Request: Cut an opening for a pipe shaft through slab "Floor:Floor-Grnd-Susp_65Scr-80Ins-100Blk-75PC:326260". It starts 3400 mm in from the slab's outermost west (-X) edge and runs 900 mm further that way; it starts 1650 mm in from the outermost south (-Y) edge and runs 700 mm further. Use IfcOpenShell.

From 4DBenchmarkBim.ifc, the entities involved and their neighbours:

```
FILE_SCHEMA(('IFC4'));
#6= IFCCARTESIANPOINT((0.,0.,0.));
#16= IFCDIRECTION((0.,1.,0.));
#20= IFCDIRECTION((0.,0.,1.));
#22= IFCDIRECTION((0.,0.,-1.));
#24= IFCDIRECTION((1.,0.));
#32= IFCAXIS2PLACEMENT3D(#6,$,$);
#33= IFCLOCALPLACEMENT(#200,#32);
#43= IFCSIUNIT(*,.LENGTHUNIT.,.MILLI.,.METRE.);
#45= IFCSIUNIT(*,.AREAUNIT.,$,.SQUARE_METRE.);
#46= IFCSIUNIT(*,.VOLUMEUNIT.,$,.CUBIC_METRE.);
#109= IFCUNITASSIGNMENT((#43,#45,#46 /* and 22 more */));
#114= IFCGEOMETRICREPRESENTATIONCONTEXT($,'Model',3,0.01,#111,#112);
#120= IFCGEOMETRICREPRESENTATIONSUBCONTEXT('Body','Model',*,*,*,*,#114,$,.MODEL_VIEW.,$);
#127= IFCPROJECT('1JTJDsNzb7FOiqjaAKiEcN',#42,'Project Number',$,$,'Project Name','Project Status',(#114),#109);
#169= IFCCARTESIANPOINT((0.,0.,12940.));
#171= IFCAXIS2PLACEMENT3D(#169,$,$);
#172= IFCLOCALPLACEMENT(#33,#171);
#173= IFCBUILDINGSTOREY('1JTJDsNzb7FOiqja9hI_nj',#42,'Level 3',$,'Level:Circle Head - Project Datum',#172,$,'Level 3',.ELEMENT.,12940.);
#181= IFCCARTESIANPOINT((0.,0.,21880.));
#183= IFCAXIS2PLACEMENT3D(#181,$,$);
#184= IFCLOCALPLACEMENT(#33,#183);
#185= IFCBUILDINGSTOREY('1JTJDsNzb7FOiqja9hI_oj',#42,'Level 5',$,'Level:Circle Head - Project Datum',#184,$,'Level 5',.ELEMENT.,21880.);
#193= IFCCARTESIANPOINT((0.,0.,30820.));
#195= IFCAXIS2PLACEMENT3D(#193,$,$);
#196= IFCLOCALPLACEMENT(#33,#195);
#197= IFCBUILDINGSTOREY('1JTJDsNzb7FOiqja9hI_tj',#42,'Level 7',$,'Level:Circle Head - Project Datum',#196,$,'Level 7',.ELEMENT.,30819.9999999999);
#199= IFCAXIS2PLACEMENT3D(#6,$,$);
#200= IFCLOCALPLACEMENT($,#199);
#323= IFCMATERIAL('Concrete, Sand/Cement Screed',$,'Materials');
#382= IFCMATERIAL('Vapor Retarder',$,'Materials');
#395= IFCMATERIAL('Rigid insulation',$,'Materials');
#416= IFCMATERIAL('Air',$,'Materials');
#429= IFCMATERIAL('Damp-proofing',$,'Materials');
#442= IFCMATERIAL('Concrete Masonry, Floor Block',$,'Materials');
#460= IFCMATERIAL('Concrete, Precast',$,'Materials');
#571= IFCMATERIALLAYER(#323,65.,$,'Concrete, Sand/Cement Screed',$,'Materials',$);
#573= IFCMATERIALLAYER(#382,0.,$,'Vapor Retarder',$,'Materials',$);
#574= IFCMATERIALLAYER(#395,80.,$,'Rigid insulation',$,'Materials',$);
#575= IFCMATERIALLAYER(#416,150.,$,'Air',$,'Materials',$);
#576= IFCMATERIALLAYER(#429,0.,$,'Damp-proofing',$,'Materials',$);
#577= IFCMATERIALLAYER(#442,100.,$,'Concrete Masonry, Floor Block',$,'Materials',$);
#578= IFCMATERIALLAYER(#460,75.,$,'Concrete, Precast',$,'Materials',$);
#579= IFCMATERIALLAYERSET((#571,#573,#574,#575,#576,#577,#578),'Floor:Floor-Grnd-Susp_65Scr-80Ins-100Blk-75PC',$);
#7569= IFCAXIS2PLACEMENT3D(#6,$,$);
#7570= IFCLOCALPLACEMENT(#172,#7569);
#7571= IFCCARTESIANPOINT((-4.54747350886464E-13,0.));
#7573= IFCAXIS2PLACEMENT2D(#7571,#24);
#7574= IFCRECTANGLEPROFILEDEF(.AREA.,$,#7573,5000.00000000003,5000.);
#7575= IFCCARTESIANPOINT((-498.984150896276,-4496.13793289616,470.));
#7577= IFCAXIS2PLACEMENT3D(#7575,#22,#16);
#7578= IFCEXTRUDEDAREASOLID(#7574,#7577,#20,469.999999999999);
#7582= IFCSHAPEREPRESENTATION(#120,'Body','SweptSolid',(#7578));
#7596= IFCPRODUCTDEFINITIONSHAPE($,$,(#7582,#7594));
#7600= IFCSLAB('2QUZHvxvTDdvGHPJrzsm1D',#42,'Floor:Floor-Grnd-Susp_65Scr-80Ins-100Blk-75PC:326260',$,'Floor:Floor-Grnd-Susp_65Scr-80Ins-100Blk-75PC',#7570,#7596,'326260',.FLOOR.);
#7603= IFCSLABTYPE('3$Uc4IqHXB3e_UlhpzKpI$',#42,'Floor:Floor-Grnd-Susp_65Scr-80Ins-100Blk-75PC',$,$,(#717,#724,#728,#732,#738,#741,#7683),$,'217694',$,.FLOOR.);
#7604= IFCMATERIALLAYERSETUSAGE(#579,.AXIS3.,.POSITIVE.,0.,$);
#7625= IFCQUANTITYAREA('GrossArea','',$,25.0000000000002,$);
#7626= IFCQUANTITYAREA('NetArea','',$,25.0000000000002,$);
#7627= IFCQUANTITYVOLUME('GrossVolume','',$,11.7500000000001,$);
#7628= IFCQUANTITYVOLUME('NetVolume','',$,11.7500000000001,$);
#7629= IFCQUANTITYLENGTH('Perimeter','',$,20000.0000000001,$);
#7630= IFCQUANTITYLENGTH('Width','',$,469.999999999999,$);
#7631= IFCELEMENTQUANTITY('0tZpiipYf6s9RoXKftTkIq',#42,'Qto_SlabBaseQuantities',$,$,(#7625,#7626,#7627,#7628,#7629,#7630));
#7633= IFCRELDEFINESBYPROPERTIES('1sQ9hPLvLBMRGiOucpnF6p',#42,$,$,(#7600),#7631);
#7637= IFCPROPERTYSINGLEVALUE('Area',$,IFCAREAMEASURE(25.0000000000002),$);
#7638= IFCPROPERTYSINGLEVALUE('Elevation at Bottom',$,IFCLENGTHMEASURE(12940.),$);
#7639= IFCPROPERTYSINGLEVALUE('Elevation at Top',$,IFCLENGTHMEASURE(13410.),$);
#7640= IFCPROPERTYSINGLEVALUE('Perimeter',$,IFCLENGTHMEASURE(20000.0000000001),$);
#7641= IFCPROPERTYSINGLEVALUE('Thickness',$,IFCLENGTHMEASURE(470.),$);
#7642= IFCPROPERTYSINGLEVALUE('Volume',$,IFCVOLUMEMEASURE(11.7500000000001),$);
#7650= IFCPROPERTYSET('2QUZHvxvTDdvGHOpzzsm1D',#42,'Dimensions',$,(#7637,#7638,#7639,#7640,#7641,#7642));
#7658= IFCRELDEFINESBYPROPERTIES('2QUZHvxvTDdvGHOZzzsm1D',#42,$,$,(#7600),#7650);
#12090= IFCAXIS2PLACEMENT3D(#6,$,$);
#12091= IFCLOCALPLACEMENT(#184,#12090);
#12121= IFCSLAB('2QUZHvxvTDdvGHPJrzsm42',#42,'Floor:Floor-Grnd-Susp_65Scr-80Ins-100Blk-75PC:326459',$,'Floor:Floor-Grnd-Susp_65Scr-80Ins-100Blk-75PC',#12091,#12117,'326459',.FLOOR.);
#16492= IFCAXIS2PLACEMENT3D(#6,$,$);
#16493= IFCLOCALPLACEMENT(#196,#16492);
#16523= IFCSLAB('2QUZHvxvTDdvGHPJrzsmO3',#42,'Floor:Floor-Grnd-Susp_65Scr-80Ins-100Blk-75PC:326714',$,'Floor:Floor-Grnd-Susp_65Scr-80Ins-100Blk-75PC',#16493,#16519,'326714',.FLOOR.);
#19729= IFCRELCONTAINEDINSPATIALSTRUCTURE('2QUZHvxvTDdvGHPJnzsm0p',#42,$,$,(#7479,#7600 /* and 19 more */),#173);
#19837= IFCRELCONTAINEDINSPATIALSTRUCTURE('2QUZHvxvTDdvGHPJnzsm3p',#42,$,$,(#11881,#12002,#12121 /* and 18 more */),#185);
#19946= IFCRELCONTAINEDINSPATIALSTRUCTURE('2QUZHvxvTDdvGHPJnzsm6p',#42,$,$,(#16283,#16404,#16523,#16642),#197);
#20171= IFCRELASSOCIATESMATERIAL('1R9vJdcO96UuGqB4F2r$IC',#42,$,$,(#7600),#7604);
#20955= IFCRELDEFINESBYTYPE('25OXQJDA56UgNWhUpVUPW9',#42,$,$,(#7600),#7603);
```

```python
import numpy as np
import ifcopenshell
import ifcopenshell.api.feature
import ifcopenshell.api.geometry
import ifcopenshell.api.pset
import ifcopenshell.api.root
import ifcopenshell.geom
import ifcopenshell.util.element
import ifcopenshell.util.placement
import ifcopenshell.util.representation
import ifcopenshell.util.shape
import ifcopenshell.util.unit

model = ifcopenshell.open("4DBenchmarkBim.ifc")
unit_scale = ifcopenshell.util.unit.calculate_unit_scale(model)
area_scale = ifcopenshell.util.unit.calculate_unit_scale(model, "AREAUNIT")
volume_scale = ifcopenshell.util.unit.calculate_unit_scale(model, "VOLUMEUNIT")
settings = ifcopenshell.geom.settings()


def volume(element):
    """Net volume in cubic metres, openings subtracted."""
    shape = ifcopenshell.geom.create_shape(settings, element)
    return ifcopenshell.util.shape.get_volume(shape.geometry)


slab = model.by_guid("2QUZHvxvTDdvGHPJrzsm1D")
before = volume(slab)

# Extent in the slab's own axes, in metres. The edges named are its -X and -Y sides.
slab_shape = ifcopenshell.geom.create_shape(settings, slab)
vertices = ifcopenshell.util.shape.get_vertices(slab_shape.geometry)
x_min, y_min, bottom = vertices.min(axis=0)
top = vertices[:, 2].max()

opening = ifcopenshell.api.root.create_entity(model, ifc_class="IfcOpeningElement", name="Pipe shaft opening", predefined_type="OPENING")
context = ifcopenshell.util.representation.get_context(model, "Model", "Body", "MODEL_VIEW")
width, depth = 0.9, 0.7
outline = [(0.0, 0.0), (width, 0.0), (width, depth), (0.0, depth), (0.0, 0.0)]
# Overshoot both faces by 50 mm so the cut is clean.
shape = ifcopenshell.api.geometry.add_slab_representation(
    model, context=context, depth=top - bottom + 0.1, polyline=outline
)
ifcopenshell.api.geometry.assign_representation(model, product=opening, representation=shape)

matrix = ifcopenshell.util.placement.get_local_placement(slab.ObjectPlacement)
matrix[:, 3] = matrix @ np.append(np.array([x_min + 3.4, y_min + 1.65, bottom - 0.05]) / unit_scale, 1.0)
ifcopenshell.api.geometry.edit_object_placement(model, product=opening, matrix=matrix, is_si=False)
ifcopenshell.api.feature.add_feature(model, feature=opening, element=slab)

after = volume(slab)

# Update the slab's stored quantities.
qto = model.by_id(ifcopenshell.util.element.get_pset(slab, "Qto_SlabBaseQuantities", should_inherit=False)["id"])
ifcopenshell.api.pset.edit_qto(model, qto=qto, properties={
    "NetArea": after / (top - bottom) / area_scale,
    "NetVolume": after / volume_scale,
})
pset = model.by_id(ifcopenshell.util.element.get_pset(slab, "Dimensions", should_inherit=False)["id"])
ifcopenshell.api.pset.edit_pset(model, pset=pset, properties={
    "Area": model.create_entity("IfcAreaMeasure", after / (top - bottom) / area_scale),
    "Volume": model.create_entity("IfcVolumeMeasure", after / volume_scale),
})

print(f"slab volume {before:.3f} -> {after:.3f} m3")

model.write("4DBenchmarkBim_edited.ifc")
```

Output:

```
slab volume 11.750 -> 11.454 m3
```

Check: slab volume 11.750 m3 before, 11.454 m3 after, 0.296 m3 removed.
